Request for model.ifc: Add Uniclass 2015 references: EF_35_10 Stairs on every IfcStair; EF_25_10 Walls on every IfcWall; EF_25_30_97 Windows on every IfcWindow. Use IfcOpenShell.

First a look at what the model holds.

```python
import ifcopenshell

model = ifcopenshell.open("model.ifc")
print(model.schema)
print("classifications:", [c.Name for c in model.by_type("IfcClassification")])
for ifc_class in ("IfcDoor", "IfcRoof", "IfcStair", "IfcWall", "IfcWindow"):
    print(ifc_class, len(model.by_type(ifc_class)))
```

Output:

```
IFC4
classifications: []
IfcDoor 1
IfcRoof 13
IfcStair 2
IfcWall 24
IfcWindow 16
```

```python
import ifcopenshell
import ifcopenshell.api.classification

model = ifcopenshell.open("model.ifc")

system = ifcopenshell.api.classification.add_classification(model, classification="Uniclass 2015")

codes = {
    "IfcStair": ("EF_35_10", "Stairs"),
    "IfcWall": ("EF_25_10", "Walls"),
    "IfcWindow": ("EF_25_30_97", "Windows"),
}
for ifc_class, (code, name) in codes.items():
    products = model.by_type(ifc_class)
    ifcopenshell.api.classification.add_reference(
        model, products=products, classification=system, identification=code, name=name
    )
    print(code, len(products))

model.write("model_rev.ifc")
```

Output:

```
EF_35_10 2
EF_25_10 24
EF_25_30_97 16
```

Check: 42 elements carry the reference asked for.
